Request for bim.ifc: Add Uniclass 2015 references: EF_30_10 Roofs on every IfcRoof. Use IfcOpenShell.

First a look at what the model holds.

```python
import ifcopenshell

model = ifcopenshell.open("bim.ifc")
print(model.schema)
print("classifications:", [c.Name for c in model.by_type("IfcClassification")])
for ifc_class in ("IfcDoor", "IfcRoof", "IfcStair", "IfcWall", "IfcWindow"):
    print(ifc_class, len(model.by_type(ifc_class)))
```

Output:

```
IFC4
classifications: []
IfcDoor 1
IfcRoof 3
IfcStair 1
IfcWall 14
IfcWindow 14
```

```python
import ifcopenshell
import ifcopenshell.api.classification

model = ifcopenshell.open("bim.ifc")

system = ifcopenshell.api.classification.add_classification(model, classification="Uniclass 2015")

codes = {
    "IfcRoof": ("EF_30_10", "Roofs"),
}
for ifc_class, (code, name) in codes.items():
    products = model.by_type(ifc_class)
    ifcopenshell.api.classification.add_reference(
        model, products=products, classification=system, identification=code, name=name
    )
    print(code, len(products))

model.write("bim_edited.ifc")
```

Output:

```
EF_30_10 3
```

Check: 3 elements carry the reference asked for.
